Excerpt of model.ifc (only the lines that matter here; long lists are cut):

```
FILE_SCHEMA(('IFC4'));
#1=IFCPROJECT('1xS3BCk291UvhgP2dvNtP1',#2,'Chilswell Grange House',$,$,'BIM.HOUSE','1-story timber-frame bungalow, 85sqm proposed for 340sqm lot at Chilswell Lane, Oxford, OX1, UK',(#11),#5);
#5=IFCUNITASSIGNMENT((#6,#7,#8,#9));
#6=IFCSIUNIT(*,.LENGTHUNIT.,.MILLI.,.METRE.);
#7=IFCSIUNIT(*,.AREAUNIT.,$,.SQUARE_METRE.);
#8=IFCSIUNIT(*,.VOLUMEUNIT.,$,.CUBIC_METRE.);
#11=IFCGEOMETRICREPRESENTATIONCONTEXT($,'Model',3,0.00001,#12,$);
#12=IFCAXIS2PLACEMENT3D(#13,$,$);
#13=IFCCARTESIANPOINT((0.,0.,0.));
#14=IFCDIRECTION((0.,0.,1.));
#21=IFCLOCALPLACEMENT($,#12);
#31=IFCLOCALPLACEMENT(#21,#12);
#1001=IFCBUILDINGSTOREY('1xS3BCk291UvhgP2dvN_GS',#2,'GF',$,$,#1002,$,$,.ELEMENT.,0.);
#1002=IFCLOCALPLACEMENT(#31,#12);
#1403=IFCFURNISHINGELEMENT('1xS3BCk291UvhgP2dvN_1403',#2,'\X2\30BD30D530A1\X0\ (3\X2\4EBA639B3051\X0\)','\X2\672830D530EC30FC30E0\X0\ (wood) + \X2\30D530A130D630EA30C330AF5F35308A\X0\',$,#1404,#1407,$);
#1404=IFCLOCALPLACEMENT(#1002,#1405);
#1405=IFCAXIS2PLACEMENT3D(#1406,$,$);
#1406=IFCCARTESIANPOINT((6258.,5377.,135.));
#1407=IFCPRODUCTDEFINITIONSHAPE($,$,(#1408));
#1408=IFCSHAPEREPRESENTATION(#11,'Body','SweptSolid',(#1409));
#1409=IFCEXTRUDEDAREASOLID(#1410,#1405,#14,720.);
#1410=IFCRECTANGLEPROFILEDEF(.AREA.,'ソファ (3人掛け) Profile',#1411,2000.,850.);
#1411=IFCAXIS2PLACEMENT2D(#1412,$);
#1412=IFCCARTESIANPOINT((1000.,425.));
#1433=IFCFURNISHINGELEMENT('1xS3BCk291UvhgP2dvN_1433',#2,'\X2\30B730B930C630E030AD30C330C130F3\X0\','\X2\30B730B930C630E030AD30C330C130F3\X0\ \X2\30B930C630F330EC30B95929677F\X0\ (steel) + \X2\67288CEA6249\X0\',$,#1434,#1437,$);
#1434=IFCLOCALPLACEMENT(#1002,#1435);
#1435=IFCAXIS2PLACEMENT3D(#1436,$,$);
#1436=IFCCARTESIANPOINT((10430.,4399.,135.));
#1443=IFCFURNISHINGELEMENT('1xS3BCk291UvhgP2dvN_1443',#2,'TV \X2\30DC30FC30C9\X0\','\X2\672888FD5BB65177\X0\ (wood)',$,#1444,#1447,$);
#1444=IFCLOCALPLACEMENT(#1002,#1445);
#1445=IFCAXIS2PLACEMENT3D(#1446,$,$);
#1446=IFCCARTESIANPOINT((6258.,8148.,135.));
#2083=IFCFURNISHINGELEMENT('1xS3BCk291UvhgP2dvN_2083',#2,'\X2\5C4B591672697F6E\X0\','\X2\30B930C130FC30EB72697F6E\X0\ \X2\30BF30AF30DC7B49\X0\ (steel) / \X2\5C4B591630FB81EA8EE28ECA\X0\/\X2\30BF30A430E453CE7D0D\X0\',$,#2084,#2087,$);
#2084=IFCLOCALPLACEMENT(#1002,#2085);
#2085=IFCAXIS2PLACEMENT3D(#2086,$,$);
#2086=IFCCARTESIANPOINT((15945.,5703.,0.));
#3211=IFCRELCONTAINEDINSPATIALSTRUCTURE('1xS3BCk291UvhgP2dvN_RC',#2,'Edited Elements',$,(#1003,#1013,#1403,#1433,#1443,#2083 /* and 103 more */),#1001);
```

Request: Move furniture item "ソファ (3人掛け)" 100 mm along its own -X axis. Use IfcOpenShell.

```python
import ifcopenshell
import ifcopenshell.api.geometry
import ifcopenshell.util.placement
import ifcopenshell.util.unit

model = ifcopenshell.open("model.ifc")
unit_scale = ifcopenshell.util.unit.calculate_unit_scale(model)

item = model.by_guid("1xS3BCk291UvhgP2dvN_1403")
matrix = ifcopenshell.util.placement.get_local_placement(item.ObjectPlacement)
matrix[:3, 3] -= matrix[:3, 0] * 0.1 / unit_scale
ifcopenshell.api.geometry.edit_object_placement(model, product=item, matrix=matrix, is_si=False)

print(ifcopenshell.util.placement.get_local_placement(item.ObjectPlacement).round(3) + 0.0)

model.write("model_updated.ifc")
```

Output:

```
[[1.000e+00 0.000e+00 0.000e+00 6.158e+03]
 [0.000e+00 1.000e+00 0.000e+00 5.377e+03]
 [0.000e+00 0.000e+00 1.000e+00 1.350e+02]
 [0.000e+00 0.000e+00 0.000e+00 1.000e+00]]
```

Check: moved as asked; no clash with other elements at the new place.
